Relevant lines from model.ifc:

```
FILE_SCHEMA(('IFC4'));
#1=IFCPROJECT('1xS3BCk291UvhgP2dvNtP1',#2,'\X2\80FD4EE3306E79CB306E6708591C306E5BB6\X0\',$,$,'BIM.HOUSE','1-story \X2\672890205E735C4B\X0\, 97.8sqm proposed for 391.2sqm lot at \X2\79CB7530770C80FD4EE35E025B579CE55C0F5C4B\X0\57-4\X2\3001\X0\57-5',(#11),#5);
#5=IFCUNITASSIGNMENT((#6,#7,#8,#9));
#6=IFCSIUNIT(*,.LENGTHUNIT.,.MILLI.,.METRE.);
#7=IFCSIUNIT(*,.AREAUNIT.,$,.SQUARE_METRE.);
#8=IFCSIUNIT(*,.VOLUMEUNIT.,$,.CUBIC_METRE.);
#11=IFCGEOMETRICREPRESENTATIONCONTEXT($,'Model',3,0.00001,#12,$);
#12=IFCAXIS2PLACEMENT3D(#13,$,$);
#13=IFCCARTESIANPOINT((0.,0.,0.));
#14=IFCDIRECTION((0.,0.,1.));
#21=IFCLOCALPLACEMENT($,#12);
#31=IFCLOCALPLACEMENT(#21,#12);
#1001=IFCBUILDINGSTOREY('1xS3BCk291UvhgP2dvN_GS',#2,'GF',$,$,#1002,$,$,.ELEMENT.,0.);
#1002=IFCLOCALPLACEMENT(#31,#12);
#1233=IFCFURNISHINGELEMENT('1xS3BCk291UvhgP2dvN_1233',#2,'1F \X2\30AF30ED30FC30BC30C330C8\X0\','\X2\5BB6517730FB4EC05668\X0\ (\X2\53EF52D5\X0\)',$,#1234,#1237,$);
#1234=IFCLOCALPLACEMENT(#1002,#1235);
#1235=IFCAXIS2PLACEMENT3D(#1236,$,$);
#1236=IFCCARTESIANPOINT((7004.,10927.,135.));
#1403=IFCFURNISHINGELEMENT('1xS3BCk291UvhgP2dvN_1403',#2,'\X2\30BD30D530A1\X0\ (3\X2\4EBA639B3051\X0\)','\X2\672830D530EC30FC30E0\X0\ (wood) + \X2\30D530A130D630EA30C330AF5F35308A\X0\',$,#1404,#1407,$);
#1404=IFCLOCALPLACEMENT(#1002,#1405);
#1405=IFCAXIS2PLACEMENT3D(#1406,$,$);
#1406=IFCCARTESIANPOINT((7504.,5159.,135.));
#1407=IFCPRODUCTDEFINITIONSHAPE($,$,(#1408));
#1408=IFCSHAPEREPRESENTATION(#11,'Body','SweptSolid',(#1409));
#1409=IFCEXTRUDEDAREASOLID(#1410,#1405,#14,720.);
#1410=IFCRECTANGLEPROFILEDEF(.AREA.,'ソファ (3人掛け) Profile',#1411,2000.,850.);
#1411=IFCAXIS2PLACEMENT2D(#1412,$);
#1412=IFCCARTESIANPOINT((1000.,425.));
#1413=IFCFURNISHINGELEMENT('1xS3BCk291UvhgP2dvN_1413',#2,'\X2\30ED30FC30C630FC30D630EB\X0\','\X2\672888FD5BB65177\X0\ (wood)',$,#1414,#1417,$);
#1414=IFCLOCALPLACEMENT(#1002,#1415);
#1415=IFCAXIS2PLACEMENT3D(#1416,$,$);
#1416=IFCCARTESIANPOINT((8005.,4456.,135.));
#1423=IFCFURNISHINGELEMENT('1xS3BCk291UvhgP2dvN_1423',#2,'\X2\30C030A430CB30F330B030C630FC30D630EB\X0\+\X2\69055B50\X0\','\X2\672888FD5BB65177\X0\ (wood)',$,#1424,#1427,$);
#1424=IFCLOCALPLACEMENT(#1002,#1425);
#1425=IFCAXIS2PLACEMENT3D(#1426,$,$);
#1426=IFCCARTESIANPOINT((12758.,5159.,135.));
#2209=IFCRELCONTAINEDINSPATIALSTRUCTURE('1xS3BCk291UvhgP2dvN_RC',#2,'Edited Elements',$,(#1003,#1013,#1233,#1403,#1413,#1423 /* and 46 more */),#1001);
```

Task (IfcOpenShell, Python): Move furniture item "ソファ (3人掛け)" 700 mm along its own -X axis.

```python
import ifcopenshell
import ifcopenshell.api.geometry
import ifcopenshell.util.placement

model = ifcopenshell.open("model.ifc")

item = model.by_id(1403)
matrix = ifcopenshell.util.placement.get_local_placement(item.ObjectPlacement)
matrix[:3, 3] -= matrix[:3, 0] * 700.0
ifcopenshell.api.geometry.edit_object_placement(model, product=item, matrix=matrix, is_si=False)

print(ifcopenshell.util.placement.get_local_placement(item.ObjectPlacement).round(3) + 0.0)

model.write("model_updated.ifc")
```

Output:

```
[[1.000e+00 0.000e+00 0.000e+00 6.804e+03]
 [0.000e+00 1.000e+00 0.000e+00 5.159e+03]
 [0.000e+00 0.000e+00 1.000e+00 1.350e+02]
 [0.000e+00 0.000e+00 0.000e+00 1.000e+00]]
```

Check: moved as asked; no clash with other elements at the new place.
